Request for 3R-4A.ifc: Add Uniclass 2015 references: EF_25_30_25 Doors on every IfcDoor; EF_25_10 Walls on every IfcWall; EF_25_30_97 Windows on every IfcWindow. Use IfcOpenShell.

First a look at what the model holds.

```python
import ifcopenshell

model = ifcopenshell.open("3R-4A.ifc")
print(model.schema)
print("classifications:", [c.Name for c in model.by_type("IfcClassification")])
for ifc_class in ("IfcDoor", "IfcRoof", "IfcStair", "IfcWall", "IfcWindow"):
    print(ifc_class, len(model.by_type(ifc_class)))
```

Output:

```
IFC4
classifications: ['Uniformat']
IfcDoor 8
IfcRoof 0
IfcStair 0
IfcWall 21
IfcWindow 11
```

```python
import ifcopenshell
import ifcopenshell.api.classification

model = ifcopenshell.open("3R-4A.ifc")

system = ifcopenshell.api.classification.add_classification(model, classification="Uniclass 2015")

codes = {
    "IfcDoor": ("EF_25_30_25", "Doors"),
    "IfcWall": ("EF_25_10", "Walls"),
    "IfcWindow": ("EF_25_30_97", "Windows"),
}
for ifc_class, (code, name) in codes.items():
    products = model.by_type(ifc_class)
    ifcopenshell.api.classification.add_reference(
        model, products=products, classification=system, identification=code, name=name
    )
    print(code, len(products))

model.write("3R-4A_rev.ifc")
```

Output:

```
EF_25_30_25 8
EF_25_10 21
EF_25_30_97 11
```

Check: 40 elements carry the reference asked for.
